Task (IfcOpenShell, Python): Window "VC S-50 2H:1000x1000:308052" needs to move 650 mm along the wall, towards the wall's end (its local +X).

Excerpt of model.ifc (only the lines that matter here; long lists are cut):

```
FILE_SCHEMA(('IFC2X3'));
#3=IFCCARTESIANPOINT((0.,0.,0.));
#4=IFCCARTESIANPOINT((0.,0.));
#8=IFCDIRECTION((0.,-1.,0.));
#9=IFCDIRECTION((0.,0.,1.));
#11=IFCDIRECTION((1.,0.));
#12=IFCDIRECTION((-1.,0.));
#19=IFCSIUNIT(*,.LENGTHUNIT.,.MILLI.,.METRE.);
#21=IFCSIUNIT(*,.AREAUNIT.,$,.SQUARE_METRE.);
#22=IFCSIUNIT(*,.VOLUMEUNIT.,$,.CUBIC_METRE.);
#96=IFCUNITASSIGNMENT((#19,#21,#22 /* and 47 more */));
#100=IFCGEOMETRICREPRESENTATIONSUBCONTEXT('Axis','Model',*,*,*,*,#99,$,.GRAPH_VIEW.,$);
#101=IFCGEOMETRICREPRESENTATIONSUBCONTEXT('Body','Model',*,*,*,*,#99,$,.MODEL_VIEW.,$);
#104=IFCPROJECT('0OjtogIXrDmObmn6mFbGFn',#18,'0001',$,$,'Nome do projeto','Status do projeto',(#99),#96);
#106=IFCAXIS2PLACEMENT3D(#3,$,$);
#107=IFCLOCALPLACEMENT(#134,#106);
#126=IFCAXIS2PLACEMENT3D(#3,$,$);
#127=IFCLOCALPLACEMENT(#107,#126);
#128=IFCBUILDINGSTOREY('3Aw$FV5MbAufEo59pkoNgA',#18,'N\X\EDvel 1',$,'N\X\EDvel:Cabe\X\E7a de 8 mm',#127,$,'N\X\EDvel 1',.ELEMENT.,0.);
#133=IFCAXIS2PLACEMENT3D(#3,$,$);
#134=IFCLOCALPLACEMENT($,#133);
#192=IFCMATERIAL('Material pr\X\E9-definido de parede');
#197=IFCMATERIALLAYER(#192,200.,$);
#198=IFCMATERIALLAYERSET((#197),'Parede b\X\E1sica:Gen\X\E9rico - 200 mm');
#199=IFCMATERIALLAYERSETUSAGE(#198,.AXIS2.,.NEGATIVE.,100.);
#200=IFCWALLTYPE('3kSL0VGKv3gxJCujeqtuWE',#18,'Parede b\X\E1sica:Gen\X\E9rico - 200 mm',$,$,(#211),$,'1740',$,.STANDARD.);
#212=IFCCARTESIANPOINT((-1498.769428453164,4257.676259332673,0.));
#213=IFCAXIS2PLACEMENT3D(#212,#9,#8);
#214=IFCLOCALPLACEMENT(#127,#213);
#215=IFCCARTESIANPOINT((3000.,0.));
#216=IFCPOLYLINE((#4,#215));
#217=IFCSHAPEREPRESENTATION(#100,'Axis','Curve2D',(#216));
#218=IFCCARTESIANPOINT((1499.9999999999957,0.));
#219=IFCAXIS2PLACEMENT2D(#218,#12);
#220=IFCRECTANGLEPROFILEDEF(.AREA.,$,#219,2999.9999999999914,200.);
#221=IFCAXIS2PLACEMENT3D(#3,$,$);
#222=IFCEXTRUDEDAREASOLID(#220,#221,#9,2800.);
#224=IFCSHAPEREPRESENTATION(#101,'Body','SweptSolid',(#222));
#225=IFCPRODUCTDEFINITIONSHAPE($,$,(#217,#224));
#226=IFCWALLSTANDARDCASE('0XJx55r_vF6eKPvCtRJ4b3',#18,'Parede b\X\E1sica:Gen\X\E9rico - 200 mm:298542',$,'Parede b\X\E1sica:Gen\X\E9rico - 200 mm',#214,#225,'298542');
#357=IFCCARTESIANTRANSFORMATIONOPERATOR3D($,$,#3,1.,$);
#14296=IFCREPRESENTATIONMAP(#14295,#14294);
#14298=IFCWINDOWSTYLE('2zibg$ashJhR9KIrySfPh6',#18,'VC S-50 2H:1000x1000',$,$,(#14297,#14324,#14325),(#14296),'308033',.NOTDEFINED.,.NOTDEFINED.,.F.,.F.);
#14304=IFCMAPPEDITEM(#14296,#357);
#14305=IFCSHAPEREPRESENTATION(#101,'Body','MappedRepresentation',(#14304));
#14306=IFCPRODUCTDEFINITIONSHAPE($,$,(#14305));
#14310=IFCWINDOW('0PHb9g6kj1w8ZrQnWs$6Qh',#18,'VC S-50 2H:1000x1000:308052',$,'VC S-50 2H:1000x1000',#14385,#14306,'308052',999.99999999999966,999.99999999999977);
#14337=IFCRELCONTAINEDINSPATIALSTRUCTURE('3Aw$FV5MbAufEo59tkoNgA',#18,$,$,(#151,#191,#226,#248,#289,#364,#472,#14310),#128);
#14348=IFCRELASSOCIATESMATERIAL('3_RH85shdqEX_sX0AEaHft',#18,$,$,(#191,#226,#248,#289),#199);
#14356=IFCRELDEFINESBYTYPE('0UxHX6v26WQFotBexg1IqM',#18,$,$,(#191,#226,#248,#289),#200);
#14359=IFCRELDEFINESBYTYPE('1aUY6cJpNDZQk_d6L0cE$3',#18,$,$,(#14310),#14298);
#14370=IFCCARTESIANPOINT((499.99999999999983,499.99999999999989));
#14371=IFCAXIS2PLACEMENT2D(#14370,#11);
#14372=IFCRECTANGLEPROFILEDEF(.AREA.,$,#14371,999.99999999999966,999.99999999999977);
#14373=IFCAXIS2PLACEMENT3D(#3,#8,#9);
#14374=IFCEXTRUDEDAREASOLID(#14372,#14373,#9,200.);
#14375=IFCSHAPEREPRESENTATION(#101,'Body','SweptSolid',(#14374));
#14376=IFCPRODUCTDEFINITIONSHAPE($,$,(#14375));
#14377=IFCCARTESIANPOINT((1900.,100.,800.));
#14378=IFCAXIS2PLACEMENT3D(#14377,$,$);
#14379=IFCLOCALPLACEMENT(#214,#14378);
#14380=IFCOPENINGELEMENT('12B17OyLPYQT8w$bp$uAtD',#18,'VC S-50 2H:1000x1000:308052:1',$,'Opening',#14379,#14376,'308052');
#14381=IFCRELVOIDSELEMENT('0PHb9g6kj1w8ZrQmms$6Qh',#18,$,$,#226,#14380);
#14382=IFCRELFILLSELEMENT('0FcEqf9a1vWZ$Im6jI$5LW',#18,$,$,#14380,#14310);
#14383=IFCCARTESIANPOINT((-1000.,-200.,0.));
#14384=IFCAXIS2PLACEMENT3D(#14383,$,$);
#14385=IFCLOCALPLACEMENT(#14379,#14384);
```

```python
import ifcopenshell
import ifcopenshell.api.geometry
import ifcopenshell.util.placement
import ifcopenshell.util.unit

model = ifcopenshell.open("model.ifc")
unit_scale = ifcopenshell.util.unit.calculate_unit_scale(model)

window = model.by_guid("0PHb9g6kj1w8ZrQnWs$6Qh")
opening = window.FillsVoids[0].RelatingOpeningElement
wall = opening.VoidsElements[0].RelatingBuildingElement

wall_matrix = ifcopenshell.util.placement.get_local_placement(wall.ObjectPlacement)
shift = wall_matrix[:3, 0] * 0.65 / unit_scale
before = ifcopenshell.util.placement.get_local_placement(window.ObjectPlacement)[:3, 3].copy()

# The window is placed relative to its opening, so it follows when the opening moves.
matrix = ifcopenshell.util.placement.get_local_placement(opening.ObjectPlacement)
matrix[:3, 3] += shift
ifcopenshell.api.geometry.edit_object_placement(
    model, product=opening, matrix=matrix, is_si=False, should_transform_children=True
)

after = ifcopenshell.util.placement.get_local_placement(window.ObjectPlacement)[:3, 3]
print("window moved by", (after - before).round(3) + 0.0)

model.write("model_v2.ifc")
```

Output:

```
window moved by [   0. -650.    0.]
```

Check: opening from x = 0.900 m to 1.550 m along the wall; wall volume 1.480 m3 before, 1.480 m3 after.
